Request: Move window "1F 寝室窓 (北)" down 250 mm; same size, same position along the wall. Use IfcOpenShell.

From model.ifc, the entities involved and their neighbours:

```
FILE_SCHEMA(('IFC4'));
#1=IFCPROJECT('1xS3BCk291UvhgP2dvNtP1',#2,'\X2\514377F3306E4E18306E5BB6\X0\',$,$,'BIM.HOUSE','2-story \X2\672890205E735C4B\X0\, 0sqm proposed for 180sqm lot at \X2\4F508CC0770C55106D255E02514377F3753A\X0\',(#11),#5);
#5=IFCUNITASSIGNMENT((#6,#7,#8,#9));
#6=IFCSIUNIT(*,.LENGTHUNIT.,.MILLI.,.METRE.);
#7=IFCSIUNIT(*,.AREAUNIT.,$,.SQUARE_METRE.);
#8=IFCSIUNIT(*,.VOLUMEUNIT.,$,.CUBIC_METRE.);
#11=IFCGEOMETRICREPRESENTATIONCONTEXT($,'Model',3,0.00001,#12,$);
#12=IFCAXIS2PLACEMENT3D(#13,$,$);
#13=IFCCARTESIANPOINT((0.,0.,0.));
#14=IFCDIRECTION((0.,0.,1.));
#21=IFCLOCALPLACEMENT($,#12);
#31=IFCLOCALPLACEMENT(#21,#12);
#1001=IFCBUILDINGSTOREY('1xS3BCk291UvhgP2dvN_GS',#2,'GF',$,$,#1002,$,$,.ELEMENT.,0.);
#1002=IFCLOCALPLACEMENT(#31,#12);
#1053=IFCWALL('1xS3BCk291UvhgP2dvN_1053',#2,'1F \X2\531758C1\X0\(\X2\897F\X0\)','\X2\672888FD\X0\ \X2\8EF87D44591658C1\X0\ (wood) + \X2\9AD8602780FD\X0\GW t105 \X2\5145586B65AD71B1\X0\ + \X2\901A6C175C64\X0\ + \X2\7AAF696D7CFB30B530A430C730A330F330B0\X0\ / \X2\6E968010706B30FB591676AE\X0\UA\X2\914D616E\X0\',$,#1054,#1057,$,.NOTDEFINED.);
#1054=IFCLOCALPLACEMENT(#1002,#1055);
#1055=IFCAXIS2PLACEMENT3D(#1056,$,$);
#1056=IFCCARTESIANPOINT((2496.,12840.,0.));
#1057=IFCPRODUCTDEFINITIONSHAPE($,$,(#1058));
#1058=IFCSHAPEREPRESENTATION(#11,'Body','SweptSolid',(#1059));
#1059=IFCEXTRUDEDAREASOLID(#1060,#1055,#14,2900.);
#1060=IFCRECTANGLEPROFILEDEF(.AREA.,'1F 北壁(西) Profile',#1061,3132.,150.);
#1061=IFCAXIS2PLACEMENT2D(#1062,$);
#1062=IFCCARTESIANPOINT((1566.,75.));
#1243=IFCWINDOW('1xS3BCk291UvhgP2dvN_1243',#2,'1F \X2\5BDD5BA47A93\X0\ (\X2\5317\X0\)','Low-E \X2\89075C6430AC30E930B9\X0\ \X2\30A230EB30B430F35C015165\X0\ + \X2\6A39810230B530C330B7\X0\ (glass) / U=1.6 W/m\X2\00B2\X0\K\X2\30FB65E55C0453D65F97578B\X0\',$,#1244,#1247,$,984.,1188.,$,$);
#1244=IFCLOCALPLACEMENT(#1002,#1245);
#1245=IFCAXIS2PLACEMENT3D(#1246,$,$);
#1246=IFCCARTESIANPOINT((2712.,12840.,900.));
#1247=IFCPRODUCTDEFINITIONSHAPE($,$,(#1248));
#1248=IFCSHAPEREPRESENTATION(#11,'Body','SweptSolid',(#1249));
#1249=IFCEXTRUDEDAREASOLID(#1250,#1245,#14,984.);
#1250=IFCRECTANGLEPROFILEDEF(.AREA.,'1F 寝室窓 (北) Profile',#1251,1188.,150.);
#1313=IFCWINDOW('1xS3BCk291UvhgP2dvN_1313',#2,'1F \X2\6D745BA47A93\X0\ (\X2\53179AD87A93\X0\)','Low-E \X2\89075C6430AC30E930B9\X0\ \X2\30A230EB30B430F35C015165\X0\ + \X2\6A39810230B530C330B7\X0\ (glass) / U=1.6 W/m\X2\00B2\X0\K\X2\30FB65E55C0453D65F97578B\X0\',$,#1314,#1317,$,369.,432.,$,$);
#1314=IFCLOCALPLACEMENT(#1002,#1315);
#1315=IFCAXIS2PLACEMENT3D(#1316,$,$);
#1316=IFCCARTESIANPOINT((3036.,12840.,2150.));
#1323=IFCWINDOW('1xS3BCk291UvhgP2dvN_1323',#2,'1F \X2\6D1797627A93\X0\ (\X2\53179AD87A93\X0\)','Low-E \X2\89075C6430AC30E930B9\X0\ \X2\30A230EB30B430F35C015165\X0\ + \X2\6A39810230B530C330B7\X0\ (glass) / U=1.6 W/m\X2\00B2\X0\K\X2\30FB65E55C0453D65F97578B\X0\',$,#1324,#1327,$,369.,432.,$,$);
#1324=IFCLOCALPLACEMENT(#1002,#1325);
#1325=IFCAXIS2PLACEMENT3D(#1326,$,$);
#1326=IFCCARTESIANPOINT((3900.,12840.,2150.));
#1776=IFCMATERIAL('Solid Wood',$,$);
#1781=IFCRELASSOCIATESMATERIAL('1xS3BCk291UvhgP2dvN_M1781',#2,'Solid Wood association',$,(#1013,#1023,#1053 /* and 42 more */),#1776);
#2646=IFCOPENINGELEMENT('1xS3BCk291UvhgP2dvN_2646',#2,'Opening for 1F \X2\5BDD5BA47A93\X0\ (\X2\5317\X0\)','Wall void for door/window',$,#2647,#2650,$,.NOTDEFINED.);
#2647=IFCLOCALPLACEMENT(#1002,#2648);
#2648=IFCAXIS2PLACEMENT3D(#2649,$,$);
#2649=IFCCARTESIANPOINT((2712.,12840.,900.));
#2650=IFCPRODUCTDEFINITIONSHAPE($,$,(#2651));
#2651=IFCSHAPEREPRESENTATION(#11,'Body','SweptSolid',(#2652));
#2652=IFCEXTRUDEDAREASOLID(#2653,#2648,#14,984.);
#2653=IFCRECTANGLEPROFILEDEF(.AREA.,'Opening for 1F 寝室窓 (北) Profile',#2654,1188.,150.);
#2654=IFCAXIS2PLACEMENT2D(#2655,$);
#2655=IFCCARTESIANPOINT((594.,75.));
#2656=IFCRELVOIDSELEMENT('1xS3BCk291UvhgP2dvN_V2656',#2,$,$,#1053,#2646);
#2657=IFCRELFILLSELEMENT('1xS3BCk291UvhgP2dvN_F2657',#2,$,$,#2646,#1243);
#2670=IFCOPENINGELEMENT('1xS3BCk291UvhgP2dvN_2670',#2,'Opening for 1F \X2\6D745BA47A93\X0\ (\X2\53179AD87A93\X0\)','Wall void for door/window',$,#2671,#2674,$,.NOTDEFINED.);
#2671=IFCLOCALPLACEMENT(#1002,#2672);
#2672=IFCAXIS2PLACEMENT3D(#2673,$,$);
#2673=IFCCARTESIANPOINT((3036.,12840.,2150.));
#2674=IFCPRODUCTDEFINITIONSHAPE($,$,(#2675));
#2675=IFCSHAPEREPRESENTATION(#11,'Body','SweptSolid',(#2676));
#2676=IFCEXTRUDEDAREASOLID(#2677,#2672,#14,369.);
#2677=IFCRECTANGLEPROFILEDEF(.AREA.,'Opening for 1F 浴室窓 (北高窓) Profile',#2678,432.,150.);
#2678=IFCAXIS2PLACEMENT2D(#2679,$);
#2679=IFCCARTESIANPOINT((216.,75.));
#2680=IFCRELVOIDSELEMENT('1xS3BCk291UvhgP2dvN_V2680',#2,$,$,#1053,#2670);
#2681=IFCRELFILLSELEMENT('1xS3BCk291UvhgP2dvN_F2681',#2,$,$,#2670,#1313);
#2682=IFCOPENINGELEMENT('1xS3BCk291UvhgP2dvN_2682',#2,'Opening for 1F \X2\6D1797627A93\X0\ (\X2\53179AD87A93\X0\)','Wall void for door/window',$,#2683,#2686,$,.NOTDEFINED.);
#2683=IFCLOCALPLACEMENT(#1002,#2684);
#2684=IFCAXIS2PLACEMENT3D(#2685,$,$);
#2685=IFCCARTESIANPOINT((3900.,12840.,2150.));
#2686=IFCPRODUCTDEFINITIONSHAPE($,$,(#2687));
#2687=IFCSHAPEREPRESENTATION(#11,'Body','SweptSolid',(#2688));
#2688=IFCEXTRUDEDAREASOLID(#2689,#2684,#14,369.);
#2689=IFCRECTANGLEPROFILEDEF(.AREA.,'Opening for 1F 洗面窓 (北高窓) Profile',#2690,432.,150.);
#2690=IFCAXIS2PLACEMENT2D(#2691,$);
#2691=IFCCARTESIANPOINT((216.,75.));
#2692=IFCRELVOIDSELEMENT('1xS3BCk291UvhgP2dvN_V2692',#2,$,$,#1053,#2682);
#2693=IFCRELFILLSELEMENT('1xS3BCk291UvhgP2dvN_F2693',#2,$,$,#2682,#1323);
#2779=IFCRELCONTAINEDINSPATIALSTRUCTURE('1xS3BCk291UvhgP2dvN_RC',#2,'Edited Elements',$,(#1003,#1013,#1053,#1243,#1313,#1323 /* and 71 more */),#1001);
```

```python
import numpy as np
import ifcopenshell
import ifcopenshell.api.geometry
import ifcopenshell.util.placement
import ifcopenshell.util.unit

model = ifcopenshell.open("model.ifc")
unit_scale = ifcopenshell.util.unit.calculate_unit_scale(model)

window = model.by_guid("1xS3BCk291UvhgP2dvN_1243")
opening = window.FillsVoids[0].RelatingOpeningElement
dz = -0.25 / unit_scale

shift = np.array([0.0, 0.0, dz])
# The window is not placed relative to its opening, so move both.
for product in (opening, window):
    matrix = ifcopenshell.util.placement.get_local_placement(product.ObjectPlacement)
    matrix[:3, 3] += shift
    ifcopenshell.api.geometry.edit_object_placement(model, product=product, matrix=matrix, is_si=False)

print(f"moved by {dz * unit_scale:+.3f} m")

model.write("model_edited.ifc")
```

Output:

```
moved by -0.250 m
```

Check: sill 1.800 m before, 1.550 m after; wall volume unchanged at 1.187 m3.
